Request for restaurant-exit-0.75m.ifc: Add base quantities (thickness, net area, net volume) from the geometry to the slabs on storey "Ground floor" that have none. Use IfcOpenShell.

First a look at what the model holds.

```python
import ifcopenshell
import ifcopenshell.util.element
import ifcopenshell.util.unit

model = ifcopenshell.open("restaurant-exit-0.75m.ifc")
print(model.schema)
for unit_type in ("LENGTHUNIT", "AREAUNIT", "VOLUMEUNIT"):
    print(unit_type, ifcopenshell.util.unit.calculate_unit_scale(model, unit_type))
storey = next(s for s in model.by_type("IfcBuildingStorey") if s.Name == "Ground floor")
slabs = [e for e in ifcopenshell.util.element.get_decomposition(storey) if e.is_a("IfcSlab")]
for e in sorted(slabs, key=lambda e: e.id()):
    print(e.id(), e.is_a(), e.Name, list(ifcopenshell.util.element.get_psets(e, qtos_only=True)), sep=" | ")
```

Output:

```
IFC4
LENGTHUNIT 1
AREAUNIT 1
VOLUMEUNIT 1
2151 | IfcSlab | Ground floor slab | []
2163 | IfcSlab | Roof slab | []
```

```python
import ifcopenshell
import ifcopenshell.api.pset
import ifcopenshell.geom
import ifcopenshell.util.element
import ifcopenshell.util.shape
import ifcopenshell.util.unit

model = ifcopenshell.open("restaurant-exit-0.75m.ifc")
unit_scale = ifcopenshell.util.unit.calculate_unit_scale(model)
area_scale = ifcopenshell.util.unit.calculate_unit_scale(model, "AREAUNIT")
volume_scale = ifcopenshell.util.unit.calculate_unit_scale(model, "VOLUMEUNIT")
settings = ifcopenshell.geom.settings()

storey = next(s for s in model.by_type("IfcBuildingStorey") if s.Name == "Ground floor")
slabs = [e for e in ifcopenshell.util.element.get_decomposition(storey) if e.is_a("IfcSlab")]

for e in sorted(slabs, key=lambda e: e.id()):
    if ifcopenshell.util.element.get_psets(e, qtos_only=True, should_inherit=False):
        continue
    # Geometry comes back in metres, in the element's own axes.
    shape = ifcopenshell.geom.create_shape(settings, e)
    values = {
        "Width": ifcopenshell.util.shape.get_z(shape.geometry) / unit_scale,
        "NetArea": ifcopenshell.util.shape.get_footprint_area(shape.geometry) / area_scale,
        "NetVolume": ifcopenshell.util.shape.get_volume(shape.geometry) / volume_scale,
    }
    qto = ifcopenshell.api.pset.add_qto(model, product=e, name="Qto_SlabBaseQuantities")
    ifcopenshell.api.pset.edit_qto(model, qto=qto, properties=values)
    print(e.id(), {k: round(v, 3) for k, v in values.items()})

model.write("restaurant-exit-0.75m_updated.ifc")
```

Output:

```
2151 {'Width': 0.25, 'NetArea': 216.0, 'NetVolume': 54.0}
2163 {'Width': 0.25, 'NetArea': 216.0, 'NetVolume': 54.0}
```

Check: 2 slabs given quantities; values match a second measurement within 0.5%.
